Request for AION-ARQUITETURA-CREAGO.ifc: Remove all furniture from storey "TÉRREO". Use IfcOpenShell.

First a look at what the model holds.

```python
import ifcopenshell
import ifcopenshell.util.element

model = ifcopenshell.open("AION-ARQUITETURA-CREAGO.ifc")
print(model.schema)
storey = next(s for s in model.by_type("IfcBuildingStorey") if s.Name == "TÉRREO")
furniture = [e for e in ifcopenshell.util.element.get_decomposition(storey) if e.is_a("IfcFurnishingElement")]
seen = {}
for e in furniture:
    element_type = ifcopenshell.util.element.get_type(e)
    name = element_type.Name if element_type not in (None, e) else None
    seen[name] = seen.get(name, 0) + 1
for name, count in sorted(seen.items(), key=str):
    print(count, "x", name)
```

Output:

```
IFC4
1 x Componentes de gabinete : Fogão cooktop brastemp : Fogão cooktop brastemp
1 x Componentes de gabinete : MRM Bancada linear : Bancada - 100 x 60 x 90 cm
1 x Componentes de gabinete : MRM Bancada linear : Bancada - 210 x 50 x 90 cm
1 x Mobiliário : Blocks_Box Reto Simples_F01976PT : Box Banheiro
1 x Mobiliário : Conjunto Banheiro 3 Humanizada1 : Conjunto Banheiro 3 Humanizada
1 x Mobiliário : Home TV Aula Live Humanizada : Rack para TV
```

```python
import ifcopenshell
import ifcopenshell.api.root
import ifcopenshell.util.element

model = ifcopenshell.open("AION-ARQUITETURA-CREAGO.ifc")

storey = next(s for s in model.by_type("IfcBuildingStorey") if s.Name == "TÉRREO")
furniture = [e for e in ifcopenshell.util.element.get_decomposition(storey) if e.is_a("IfcFurnishingElement")]

for e in furniture:
    ifcopenshell.api.root.remove_product(model, product=e)
print(len(furniture), "removed")

model.write("AION-ARQUITETURA-CREAGO_v2.ifc")
```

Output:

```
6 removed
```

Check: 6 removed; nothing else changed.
